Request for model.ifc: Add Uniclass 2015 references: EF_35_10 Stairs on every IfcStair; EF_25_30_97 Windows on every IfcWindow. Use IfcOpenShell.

First a look at what the model holds.

```python
import ifcopenshell

model = ifcopenshell.open("model.ifc")
print(model.schema)
print("classifications:", [c.Name for c in model.by_type("IfcClassification")])
for ifc_class in ("IfcDoor", "IfcRoof", "IfcStair", "IfcWall", "IfcWindow"):
    print(ifc_class, len(model.by_type(ifc_class)))
```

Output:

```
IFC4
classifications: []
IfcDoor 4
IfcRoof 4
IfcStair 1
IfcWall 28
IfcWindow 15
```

```python
import ifcopenshell
import ifcopenshell.api.classification

model = ifcopenshell.open("model.ifc")

system = ifcopenshell.api.classification.add_classification(model, classification="Uniclass 2015")

codes = {
    "IfcStair": ("EF_35_10", "Stairs"),
    "IfcWindow": ("EF_25_30_97", "Windows"),
}
for ifc_class, (code, name) in codes.items():
    products = model.by_type(ifc_class)
    ifcopenshell.api.classification.add_reference(
        model, products=products, classification=system, identification=code, name=name
    )
    print(code, len(products))

model.write("model_rev.ifc")
```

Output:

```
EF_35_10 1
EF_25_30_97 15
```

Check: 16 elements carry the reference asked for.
